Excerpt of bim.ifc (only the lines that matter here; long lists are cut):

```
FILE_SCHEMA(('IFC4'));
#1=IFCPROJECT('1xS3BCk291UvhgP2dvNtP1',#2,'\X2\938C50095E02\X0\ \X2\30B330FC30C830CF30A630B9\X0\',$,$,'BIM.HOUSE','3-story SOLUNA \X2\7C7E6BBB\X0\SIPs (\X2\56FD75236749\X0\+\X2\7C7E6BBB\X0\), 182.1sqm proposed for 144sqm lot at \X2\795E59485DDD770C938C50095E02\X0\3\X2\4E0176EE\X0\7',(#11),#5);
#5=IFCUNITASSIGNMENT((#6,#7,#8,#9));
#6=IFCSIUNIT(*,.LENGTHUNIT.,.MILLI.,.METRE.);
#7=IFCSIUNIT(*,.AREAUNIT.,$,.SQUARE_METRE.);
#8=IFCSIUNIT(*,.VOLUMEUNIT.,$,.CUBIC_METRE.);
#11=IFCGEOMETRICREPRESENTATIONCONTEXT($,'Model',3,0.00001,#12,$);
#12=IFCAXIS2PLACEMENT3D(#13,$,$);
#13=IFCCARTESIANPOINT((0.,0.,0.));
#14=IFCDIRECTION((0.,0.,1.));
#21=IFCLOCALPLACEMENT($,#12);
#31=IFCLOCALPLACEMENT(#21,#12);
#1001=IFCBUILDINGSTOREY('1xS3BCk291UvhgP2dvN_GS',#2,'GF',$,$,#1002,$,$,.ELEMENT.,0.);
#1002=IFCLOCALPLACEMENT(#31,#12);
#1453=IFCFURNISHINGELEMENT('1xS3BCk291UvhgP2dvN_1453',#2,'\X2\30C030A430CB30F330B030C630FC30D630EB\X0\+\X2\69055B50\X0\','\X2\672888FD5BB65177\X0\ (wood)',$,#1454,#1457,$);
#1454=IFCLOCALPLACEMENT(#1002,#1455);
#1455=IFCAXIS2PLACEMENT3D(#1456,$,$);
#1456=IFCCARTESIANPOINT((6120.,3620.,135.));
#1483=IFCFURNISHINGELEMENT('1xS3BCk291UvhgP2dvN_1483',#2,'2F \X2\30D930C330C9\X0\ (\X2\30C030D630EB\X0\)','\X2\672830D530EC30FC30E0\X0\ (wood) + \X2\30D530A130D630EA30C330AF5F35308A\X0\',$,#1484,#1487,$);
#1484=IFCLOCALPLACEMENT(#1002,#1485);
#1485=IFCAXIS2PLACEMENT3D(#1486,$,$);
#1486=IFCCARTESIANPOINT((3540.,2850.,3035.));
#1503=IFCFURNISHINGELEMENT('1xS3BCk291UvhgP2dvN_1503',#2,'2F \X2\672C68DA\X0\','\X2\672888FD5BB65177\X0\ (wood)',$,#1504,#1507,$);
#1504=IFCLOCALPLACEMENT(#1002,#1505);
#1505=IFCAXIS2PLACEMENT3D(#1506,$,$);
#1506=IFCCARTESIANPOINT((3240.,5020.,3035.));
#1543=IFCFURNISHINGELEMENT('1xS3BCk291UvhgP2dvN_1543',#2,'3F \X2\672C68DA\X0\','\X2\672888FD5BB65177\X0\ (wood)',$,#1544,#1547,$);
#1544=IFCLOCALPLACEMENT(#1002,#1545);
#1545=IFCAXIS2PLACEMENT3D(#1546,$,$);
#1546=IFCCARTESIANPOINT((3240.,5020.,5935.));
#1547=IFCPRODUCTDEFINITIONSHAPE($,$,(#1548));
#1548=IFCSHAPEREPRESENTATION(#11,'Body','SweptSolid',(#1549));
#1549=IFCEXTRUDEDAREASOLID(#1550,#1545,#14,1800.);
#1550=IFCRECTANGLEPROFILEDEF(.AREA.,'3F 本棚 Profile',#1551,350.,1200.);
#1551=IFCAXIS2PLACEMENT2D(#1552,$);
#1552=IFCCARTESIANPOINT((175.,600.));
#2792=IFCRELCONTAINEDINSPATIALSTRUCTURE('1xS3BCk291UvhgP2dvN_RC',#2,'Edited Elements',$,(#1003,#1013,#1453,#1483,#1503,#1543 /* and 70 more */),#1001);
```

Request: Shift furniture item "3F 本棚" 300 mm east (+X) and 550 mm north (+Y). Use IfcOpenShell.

```python
import ifcopenshell
import ifcopenshell.api.geometry
import ifcopenshell.util.placement
import ifcopenshell.util.unit

model = ifcopenshell.open("bim.ifc")
unit_scale = ifcopenshell.util.unit.calculate_unit_scale(model)

item = model.by_guid("1xS3BCk291UvhgP2dvN_1543")
matrix = ifcopenshell.util.placement.get_local_placement(item.ObjectPlacement)
matrix[0, 3] += 0.3 / unit_scale
matrix[1, 3] += 0.55 / unit_scale
ifcopenshell.api.geometry.edit_object_placement(model, product=item, matrix=matrix, is_si=False)

print(ifcopenshell.util.placement.get_local_placement(item.ObjectPlacement).round(3) + 0.0)

model.write("bim-out.ifc")
```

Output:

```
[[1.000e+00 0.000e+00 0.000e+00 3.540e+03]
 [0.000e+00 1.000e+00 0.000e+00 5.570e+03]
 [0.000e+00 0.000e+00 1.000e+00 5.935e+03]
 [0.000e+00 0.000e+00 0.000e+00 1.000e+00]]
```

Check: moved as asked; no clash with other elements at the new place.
